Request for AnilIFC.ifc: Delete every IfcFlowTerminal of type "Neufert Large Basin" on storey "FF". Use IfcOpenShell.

First a look at what the model holds.

```python
import ifcopenshell
import ifcopenshell.util.element

model = ifcopenshell.open("AnilIFC.ifc")
print(model.schema)
storey = next(s for s in model.by_type("IfcBuildingStorey") if s.Name == "FF")
terminals = [e for e in ifcopenshell.util.element.get_decomposition(storey) if e.is_a("IfcFlowTerminal")]
seen = {}
for e in terminals:
    element_type = ifcopenshell.util.element.get_type(e)
    name = element_type.Name if element_type not in (None, e) else None
    seen[name] = seen.get(name, 0) + 1
for name, count in sorted(seen.items(), key=str):
    print(count, "x", name)
```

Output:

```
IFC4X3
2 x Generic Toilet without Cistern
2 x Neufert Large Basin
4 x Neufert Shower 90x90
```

```python
import ifcopenshell
import ifcopenshell.api.root
import ifcopenshell.util.element

model = ifcopenshell.open("AnilIFC.ifc")

storey = next(s for s in model.by_type("IfcBuildingStorey") if s.Name == "FF")
terminals = [e for e in ifcopenshell.util.element.get_decomposition(storey) if e.is_a("IfcFlowTerminal")]
targets = [e for e in terminals if (t := ifcopenshell.util.element.get_type(e)) not in (None, e) and t.Name == "Neufert Large Basin"]

for e in targets:
    ifcopenshell.api.root.remove_product(model, product=e)
print(len(targets), "removed")

model.write("AnilIFC_v2.ifc")
```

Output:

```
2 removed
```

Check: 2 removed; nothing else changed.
